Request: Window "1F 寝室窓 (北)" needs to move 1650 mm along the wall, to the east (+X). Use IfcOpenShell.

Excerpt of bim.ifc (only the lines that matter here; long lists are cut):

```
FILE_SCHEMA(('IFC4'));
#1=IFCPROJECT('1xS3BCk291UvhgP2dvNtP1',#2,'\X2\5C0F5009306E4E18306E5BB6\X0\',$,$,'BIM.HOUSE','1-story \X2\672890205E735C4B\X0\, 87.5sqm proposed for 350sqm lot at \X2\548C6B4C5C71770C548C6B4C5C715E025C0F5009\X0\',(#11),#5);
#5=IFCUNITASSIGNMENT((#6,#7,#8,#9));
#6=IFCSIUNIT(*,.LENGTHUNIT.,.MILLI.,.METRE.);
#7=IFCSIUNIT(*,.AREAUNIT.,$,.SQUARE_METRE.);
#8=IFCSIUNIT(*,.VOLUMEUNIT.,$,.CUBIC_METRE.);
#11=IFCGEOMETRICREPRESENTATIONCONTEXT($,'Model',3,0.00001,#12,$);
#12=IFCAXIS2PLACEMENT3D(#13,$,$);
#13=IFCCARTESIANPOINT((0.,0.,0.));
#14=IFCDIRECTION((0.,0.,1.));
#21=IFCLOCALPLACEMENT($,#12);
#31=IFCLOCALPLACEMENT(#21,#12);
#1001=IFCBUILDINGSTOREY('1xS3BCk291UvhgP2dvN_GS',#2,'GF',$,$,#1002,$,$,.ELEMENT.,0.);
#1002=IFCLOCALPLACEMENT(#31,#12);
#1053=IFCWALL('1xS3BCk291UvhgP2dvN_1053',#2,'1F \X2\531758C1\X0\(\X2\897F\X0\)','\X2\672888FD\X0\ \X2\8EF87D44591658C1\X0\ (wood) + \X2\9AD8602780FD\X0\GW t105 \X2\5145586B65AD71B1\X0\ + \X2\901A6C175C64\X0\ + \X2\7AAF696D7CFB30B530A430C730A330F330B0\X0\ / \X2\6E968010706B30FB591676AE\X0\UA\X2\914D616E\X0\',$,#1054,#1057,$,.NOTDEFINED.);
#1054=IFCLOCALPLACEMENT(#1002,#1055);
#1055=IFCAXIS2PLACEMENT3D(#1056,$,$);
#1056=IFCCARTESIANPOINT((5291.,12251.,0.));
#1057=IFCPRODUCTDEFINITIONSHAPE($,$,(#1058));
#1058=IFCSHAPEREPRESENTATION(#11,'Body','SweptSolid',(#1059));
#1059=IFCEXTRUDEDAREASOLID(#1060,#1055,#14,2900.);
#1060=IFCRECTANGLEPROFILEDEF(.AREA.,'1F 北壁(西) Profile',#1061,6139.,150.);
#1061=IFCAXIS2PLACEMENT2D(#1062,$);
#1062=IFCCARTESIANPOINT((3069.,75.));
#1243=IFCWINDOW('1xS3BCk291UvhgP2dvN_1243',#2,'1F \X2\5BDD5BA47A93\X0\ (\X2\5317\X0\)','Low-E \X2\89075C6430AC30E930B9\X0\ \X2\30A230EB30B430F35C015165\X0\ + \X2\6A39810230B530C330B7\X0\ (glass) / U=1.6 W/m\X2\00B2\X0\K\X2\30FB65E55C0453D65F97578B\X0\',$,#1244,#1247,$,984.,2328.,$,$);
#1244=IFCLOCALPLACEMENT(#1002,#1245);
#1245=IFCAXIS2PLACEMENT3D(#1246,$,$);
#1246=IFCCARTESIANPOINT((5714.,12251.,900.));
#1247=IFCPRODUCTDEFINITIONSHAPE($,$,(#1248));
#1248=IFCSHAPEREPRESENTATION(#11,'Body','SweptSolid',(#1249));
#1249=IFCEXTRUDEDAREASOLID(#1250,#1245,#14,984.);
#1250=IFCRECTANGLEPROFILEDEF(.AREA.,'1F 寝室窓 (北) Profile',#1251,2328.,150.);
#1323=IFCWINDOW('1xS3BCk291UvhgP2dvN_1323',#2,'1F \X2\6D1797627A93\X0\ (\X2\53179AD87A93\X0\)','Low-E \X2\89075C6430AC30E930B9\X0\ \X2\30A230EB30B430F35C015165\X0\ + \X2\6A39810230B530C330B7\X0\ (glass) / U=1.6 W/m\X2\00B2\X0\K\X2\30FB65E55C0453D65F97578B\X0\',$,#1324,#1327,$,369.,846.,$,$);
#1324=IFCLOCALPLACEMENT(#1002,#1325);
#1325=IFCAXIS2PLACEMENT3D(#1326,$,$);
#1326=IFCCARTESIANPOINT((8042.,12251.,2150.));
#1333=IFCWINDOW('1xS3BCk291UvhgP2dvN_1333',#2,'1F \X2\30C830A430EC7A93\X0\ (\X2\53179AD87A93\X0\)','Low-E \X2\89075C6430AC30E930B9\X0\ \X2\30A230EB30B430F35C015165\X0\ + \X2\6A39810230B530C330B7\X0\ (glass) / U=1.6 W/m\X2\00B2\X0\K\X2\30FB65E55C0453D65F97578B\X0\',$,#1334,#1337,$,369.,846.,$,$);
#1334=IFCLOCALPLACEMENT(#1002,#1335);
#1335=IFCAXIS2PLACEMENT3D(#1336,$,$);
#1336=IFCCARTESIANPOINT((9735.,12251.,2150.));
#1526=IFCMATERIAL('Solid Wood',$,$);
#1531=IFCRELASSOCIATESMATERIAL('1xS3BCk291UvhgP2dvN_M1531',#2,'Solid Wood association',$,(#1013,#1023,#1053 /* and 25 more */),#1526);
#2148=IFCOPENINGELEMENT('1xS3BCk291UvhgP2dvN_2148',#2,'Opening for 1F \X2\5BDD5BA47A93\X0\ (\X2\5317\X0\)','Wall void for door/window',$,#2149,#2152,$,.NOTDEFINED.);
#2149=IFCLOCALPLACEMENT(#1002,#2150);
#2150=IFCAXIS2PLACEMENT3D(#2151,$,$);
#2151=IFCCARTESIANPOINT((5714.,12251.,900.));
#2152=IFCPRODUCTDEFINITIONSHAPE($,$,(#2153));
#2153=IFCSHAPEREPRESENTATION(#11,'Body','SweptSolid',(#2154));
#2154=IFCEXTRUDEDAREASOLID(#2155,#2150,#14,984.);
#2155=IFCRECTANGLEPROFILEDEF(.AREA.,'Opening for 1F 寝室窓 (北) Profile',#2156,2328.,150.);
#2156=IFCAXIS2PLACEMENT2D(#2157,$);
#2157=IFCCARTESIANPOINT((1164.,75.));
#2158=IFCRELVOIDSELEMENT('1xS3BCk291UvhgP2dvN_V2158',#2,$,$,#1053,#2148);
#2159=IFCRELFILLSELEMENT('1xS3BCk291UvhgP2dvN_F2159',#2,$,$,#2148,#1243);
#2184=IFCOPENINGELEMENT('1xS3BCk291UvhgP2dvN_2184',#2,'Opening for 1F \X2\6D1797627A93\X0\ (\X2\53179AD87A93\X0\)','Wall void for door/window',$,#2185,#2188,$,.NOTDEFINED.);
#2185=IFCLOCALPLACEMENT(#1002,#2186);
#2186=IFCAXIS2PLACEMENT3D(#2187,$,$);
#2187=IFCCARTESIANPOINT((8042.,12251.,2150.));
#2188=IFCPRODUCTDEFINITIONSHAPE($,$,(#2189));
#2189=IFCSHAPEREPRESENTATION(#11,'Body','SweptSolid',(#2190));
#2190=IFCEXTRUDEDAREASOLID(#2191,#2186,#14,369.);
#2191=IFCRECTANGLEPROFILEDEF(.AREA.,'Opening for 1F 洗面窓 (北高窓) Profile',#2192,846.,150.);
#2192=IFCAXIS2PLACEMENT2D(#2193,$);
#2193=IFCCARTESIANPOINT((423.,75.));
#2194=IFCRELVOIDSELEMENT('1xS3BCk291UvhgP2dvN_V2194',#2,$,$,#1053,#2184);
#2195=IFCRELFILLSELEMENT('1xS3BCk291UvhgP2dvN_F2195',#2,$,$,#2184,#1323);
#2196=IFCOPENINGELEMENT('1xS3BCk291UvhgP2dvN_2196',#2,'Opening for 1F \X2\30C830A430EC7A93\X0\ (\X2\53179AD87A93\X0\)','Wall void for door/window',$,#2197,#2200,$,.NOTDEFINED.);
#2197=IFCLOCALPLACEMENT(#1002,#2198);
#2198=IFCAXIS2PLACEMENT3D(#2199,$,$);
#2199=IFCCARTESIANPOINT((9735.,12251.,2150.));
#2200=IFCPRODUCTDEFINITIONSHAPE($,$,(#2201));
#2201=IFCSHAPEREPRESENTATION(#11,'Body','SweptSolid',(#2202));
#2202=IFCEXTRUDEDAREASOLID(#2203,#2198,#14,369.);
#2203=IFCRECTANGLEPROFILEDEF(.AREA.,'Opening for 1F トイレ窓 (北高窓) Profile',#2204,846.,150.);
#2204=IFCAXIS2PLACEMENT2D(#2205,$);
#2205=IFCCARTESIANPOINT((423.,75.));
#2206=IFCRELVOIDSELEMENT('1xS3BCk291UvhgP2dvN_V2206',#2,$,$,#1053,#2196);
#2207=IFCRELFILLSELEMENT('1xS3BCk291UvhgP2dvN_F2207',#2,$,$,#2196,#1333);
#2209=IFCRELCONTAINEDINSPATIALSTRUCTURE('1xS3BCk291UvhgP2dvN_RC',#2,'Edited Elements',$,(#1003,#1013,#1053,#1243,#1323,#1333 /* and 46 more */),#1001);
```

```python
import ifcopenshell
import ifcopenshell.api.geometry
import ifcopenshell.util.placement
import ifcopenshell.util.unit

model = ifcopenshell.open("bim.ifc")
unit_scale = ifcopenshell.util.unit.calculate_unit_scale(model)

window = model.by_guid("1xS3BCk291UvhgP2dvN_1243")
opening = window.FillsVoids[0].RelatingOpeningElement
wall = opening.VoidsElements[0].RelatingBuildingElement

wall_matrix = ifcopenshell.util.placement.get_local_placement(wall.ObjectPlacement)
shift = wall_matrix[:3, 0] * 1.65 / unit_scale
before = ifcopenshell.util.placement.get_local_placement(window.ObjectPlacement)[:3, 3].copy()

# The window is not placed relative to its opening, so move both.
for product in (opening, window):
    matrix = ifcopenshell.util.placement.get_local_placement(product.ObjectPlacement)
    matrix[:3, 3] += shift
    ifcopenshell.api.geometry.edit_object_placement(model, product=product, matrix=matrix, is_si=False)

after = ifcopenshell.util.placement.get_local_placement(window.ObjectPlacement)[:3, 3]
print("window moved by", (after - before).round(3) + 0.0)

model.write("bim_edited.ifc")
```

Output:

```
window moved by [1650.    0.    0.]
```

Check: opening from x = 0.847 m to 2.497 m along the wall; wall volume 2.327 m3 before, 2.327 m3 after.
